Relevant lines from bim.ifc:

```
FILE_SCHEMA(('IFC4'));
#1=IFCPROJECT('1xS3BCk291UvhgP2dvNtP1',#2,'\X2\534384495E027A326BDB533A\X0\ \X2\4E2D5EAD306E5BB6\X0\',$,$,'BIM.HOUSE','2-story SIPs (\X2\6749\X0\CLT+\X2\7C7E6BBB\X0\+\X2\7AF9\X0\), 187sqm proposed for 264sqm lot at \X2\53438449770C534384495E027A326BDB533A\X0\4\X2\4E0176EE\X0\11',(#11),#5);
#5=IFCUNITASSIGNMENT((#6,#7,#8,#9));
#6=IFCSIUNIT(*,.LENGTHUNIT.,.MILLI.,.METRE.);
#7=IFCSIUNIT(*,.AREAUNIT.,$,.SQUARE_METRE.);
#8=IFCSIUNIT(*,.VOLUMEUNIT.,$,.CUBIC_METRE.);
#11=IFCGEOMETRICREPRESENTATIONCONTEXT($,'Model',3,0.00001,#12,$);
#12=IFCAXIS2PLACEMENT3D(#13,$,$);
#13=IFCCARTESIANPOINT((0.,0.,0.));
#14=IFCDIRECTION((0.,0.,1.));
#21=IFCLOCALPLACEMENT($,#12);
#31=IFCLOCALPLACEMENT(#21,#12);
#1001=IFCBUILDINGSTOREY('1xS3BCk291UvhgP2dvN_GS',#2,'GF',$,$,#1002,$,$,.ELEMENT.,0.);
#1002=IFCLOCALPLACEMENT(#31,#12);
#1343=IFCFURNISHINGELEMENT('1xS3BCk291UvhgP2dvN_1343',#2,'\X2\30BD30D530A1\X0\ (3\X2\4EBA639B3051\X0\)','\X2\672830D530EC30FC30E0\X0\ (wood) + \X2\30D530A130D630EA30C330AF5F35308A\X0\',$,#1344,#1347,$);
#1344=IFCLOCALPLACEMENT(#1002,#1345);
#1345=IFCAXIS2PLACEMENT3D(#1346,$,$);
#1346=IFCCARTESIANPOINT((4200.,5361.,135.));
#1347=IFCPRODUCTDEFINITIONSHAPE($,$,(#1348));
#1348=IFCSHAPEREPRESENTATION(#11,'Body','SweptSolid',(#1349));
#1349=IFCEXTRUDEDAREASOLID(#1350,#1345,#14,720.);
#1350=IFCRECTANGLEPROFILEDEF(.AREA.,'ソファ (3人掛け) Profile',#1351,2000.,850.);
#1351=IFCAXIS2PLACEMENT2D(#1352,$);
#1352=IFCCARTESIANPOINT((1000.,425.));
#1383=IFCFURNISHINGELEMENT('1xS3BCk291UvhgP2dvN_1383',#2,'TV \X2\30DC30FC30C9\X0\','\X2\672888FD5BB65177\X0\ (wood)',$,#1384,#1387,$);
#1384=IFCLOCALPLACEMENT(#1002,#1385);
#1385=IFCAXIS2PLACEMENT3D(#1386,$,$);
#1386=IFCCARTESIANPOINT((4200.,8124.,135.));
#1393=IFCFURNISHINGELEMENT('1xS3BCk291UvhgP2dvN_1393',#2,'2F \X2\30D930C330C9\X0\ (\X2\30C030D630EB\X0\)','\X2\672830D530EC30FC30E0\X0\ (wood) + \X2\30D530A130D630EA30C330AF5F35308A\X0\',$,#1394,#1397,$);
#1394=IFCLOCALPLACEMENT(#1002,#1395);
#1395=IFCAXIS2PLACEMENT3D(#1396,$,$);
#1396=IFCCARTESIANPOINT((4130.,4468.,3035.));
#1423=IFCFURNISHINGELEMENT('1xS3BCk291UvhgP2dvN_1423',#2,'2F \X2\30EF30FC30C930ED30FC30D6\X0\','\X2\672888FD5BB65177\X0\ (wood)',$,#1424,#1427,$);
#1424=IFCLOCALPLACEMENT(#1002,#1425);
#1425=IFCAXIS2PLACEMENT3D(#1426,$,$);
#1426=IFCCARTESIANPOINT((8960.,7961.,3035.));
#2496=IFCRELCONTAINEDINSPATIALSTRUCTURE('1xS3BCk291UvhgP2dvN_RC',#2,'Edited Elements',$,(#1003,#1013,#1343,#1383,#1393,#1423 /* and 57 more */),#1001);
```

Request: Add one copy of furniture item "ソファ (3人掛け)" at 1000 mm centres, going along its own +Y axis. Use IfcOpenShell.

```python
import ifcopenshell
import ifcopenshell.api.geometry
import ifcopenshell.api.root
import ifcopenshell.util.element
import ifcopenshell.util.placement

model = ifcopenshell.open("bim.ifc")


def reuse_history(source, copy):
    """copy_class also copies each property set's owner history, people and application; keep the originals."""
    for rel in copy.IsDefinedBy:
        if rel.is_a("IfcRelDefinesByProperties") and (history := rel.RelatingPropertyDefinition.OwnerHistory):
            rel.RelatingPropertyDefinition.OwnerHistory = source.OwnerHistory
            ifcopenshell.util.element.remove_deep2(model, history)


source = model.by_guid("1xS3BCk291UvhgP2dvN_1343")
base = ifcopenshell.util.placement.get_local_placement(source.ObjectPlacement)
step = base[:3, 1] * 1000.0

for i in range(1, 2):
    copy = ifcopenshell.api.root.copy_class(model, product=source)
    copy.Representation = ifcopenshell.util.element.copy_deep(
        model, source.Representation, exclude=["IfcGeometricRepresentationContext", "IfcRepresentationMap"]
    )
    reuse_history(source, copy)
    matrix = base.copy()
    matrix[:3, 3] += i * step
    print("added at", matrix[:3, 3].round(3) + 0.0)
    ifcopenshell.api.geometry.edit_object_placement(model, product=copy, matrix=matrix, is_si=False)

model.write("bim_edited.ifc")
```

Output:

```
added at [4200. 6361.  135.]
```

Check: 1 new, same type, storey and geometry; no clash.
